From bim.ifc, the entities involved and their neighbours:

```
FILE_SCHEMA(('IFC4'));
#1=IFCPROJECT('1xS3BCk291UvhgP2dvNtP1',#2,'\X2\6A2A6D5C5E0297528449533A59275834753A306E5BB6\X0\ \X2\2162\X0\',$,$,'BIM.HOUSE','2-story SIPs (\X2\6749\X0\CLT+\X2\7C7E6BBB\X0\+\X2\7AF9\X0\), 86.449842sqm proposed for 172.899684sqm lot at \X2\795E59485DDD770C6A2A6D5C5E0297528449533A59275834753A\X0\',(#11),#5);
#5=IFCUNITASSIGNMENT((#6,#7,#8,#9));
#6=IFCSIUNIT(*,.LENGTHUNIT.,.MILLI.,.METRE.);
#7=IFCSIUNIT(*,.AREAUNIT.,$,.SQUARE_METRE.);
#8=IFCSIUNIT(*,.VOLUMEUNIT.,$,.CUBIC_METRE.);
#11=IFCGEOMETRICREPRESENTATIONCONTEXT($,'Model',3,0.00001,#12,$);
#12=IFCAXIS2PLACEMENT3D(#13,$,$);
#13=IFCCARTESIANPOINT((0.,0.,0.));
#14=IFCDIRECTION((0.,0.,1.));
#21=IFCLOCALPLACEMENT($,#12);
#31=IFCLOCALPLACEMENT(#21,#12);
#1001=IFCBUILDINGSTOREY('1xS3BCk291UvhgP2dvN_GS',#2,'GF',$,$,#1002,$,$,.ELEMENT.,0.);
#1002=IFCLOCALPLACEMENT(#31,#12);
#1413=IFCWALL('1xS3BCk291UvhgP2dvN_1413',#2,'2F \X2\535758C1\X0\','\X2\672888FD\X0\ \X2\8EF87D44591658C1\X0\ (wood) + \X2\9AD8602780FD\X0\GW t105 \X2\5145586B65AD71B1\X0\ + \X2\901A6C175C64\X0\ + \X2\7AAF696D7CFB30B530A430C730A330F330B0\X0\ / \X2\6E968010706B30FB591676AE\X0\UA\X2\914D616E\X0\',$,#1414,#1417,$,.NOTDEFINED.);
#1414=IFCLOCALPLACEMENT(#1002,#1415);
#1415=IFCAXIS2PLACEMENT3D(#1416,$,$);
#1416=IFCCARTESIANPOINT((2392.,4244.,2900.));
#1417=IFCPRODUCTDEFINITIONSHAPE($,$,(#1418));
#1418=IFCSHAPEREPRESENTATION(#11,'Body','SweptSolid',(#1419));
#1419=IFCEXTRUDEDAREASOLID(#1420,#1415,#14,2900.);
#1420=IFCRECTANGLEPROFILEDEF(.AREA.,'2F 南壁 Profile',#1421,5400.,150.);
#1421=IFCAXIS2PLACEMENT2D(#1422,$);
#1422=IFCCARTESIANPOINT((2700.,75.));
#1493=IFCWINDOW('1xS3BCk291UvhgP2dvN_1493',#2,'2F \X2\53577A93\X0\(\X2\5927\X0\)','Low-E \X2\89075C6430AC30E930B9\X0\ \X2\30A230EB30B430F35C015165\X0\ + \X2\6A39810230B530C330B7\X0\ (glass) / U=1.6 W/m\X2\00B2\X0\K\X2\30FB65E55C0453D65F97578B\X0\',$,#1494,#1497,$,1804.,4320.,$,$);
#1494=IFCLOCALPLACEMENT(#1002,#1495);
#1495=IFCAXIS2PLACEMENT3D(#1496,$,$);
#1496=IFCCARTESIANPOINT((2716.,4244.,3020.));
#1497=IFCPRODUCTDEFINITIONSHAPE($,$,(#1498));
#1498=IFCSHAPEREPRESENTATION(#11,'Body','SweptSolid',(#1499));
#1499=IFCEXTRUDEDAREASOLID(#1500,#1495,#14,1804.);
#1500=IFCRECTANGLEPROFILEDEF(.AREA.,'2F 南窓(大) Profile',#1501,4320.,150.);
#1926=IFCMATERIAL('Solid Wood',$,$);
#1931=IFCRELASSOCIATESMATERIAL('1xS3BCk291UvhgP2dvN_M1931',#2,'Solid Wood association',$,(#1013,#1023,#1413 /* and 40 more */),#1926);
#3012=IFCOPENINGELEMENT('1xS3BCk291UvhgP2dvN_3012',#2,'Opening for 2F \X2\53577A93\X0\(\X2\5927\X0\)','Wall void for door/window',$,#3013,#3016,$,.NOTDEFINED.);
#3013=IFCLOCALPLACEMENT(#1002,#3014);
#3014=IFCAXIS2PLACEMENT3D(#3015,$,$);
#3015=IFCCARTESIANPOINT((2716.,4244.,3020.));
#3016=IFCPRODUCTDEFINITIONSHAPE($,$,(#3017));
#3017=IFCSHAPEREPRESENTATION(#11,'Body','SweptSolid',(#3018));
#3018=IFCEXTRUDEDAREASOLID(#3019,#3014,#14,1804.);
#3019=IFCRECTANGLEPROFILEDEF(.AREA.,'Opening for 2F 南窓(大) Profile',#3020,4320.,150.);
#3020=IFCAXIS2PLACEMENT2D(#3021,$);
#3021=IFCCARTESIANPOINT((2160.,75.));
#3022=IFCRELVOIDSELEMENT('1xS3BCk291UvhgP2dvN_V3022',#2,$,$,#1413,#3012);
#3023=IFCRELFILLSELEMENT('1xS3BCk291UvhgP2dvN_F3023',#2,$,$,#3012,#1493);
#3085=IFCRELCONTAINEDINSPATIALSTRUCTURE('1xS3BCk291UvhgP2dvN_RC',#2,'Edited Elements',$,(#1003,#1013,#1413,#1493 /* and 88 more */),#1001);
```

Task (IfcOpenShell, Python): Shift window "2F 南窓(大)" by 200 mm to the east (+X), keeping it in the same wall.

```python
import ifcopenshell
import ifcopenshell.api.geometry
import ifcopenshell.util.placement

model = ifcopenshell.open("bim.ifc")

window = model.by_guid("1xS3BCk291UvhgP2dvN_1493")
opening = window.FillsVoids[0].RelatingOpeningElement
wall = opening.VoidsElements[0].RelatingBuildingElement

wall_matrix = ifcopenshell.util.placement.get_local_placement(wall.ObjectPlacement)
shift = wall_matrix[:3, 0] * 200.0
before = ifcopenshell.util.placement.get_local_placement(window.ObjectPlacement)[:3, 3].copy()

# The window is not placed relative to its opening, so move both.
for product in (opening, window):
    matrix = ifcopenshell.util.placement.get_local_placement(product.ObjectPlacement)
    matrix[:3, 3] += shift
    ifcopenshell.api.geometry.edit_object_placement(model, product=product, matrix=matrix, is_si=False)

after = ifcopenshell.util.placement.get_local_placement(window.ObjectPlacement)[:3, 3]
print("window moved by", (after - before).round(3) + 0.0)

model.write("bim_updated.ifc")
```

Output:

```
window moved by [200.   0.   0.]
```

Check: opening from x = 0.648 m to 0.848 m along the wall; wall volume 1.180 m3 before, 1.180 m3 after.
